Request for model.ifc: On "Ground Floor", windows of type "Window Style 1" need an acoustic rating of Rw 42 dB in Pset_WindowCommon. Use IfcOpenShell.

First a look at what the model holds.

```python
import ifcopenshell
import ifcopenshell.util.element

model = ifcopenshell.open("model.ifc")
print(model.schema)
storey = next(s for s in model.by_type("IfcBuildingStorey") if s.Name == "Ground Floor")
windows = [e for e in ifcopenshell.util.element.get_decomposition(storey) if e.is_a("IfcWindow")]
seen = {}
for e in windows:
    element_type = ifcopenshell.util.element.get_type(e)
    key = (element_type.Name if element_type != e and element_type else None, ifcopenshell.util.element.get_pset(e, "Pset_WindowCommon", "AcousticRating"))
    seen[key] = seen.get(key, 0) + 1
for (name, value), count in sorted(seen.items(), key=str):
    print(count, "x", name, "|", value)
```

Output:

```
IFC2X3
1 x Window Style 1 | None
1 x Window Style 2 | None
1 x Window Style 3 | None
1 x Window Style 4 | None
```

```python
import ifcopenshell
import ifcopenshell.api.pset
import ifcopenshell.util.element

model = ifcopenshell.open("model.ifc")

storey = next(s for s in model.by_type("IfcBuildingStorey") if s.Name == "Ground Floor")
windows = [e for e in ifcopenshell.util.element.get_decomposition(storey) if e.is_a("IfcWindow")]

count = 0
for e in windows:
    element_type = ifcopenshell.util.element.get_type(e)
    if element_type in (None, e) or element_type.Name != "Window Style 1":
        continue
    # add_pset returns the element's existing set when there is one.
    pset = ifcopenshell.api.pset.add_pset(model, product=e, name="Pset_WindowCommon")
    ifcopenshell.api.pset.edit_pset(model, pset=pset, properties={"AcousticRating": "Rw 42 dB"})
    count += 1

print(count, "windows updated")

model.write("model_updated.ifc")
```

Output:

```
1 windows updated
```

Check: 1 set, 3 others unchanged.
